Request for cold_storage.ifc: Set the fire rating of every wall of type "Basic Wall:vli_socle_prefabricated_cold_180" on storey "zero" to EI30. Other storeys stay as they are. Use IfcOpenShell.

First a look at what the model holds.

```python
import ifcopenshell
import ifcopenshell.util.element

model = ifcopenshell.open("cold_storage.ifc")
print(model.schema)
storey = next(s for s in model.by_type("IfcBuildingStorey") if s.Name == "zero")
walls = [e for e in ifcopenshell.util.element.get_decomposition(storey) if e.is_a("IfcWall")]
seen = {}
for e in walls:
    element_type = ifcopenshell.util.element.get_type(e)
    key = (element_type.Name if element_type != e and element_type else None, ifcopenshell.util.element.get_pset(e, "Pset_WallCommon", "FireRating"))
    seen[key] = seen.get(key, 0) + 1
for (name, value), count in sorted(seen.items(), key=str):
    print(count, "x", name, "|", value)
```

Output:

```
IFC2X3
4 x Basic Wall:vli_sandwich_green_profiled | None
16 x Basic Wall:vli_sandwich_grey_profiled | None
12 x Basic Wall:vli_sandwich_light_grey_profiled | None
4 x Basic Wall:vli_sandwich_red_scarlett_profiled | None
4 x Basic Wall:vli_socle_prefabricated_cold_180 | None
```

```python
import ifcopenshell
import ifcopenshell.api.pset
import ifcopenshell.util.element

model = ifcopenshell.open("cold_storage.ifc")

storey = next(s for s in model.by_type("IfcBuildingStorey") if s.Name == "zero")
walls = [e for e in ifcopenshell.util.element.get_decomposition(storey) if e.is_a("IfcWall")]

count = 0
for e in walls:
    element_type = ifcopenshell.util.element.get_type(e)
    if element_type in (None, e) or element_type.Name != "Basic Wall:vli_socle_prefabricated_cold_180":
        continue
    # add_pset returns the element's existing set when there is one.
    pset = ifcopenshell.api.pset.add_pset(model, product=e, name="Pset_WallCommon")
    ifcopenshell.api.pset.edit_pset(model, pset=pset, properties={"FireRating": "EI30"})
    count += 1

print(count, "walls updated")

model.write("cold_storage_v2.ifc")
```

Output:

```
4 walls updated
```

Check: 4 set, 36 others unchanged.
